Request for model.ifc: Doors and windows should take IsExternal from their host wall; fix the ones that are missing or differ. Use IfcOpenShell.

First a look at what the model holds.

```python
import ifcopenshell
import ifcopenshell.util.element

model = ifcopenshell.open("model.ifc")
print(model.schema)
seen = {}
for e in model.by_type("IfcDoor") + model.by_type("IfcWindow"):
    if not e.FillsVoids:
        continue
    host = e.FillsVoids[0].RelatingOpeningElement.VoidsElements[0].RelatingBuildingElement
    own = ifcopenshell.util.element.get_pset(e, f"Pset_{e.is_a()[3:].removesuffix('StandardCase')}Common", "IsExternal")
    wall = ifcopenshell.util.element.get_pset(host, "Pset_WallCommon", "IsExternal")
    seen[e.is_a(), own, wall] = seen.get((e.is_a(), own, wall), 0) + 1
for (cls, own, wall), count in sorted(seen.items(), key=str):
    print(count, cls, "IsExternal:", own, "| host wall:", wall)
```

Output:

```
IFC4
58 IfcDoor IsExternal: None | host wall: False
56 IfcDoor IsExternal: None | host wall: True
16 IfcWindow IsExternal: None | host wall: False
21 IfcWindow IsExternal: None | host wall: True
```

```python
import ifcopenshell
import ifcopenshell.api.pset
import ifcopenshell.util.element

model = ifcopenshell.open("model.ifc")

count = 0
for ifc_class, pset_name in (("IfcDoor", "Pset_DoorCommon"), ("IfcWindow", "Pset_WindowCommon")):
    for e in model.by_type(ifc_class):
        if not e.FillsVoids:
            continue
        host = e.FillsVoids[0].RelatingOpeningElement.VoidsElements[0].RelatingBuildingElement
        external = ifcopenshell.util.element.get_pset(host, "Pset_WallCommon", "IsExternal")
        if external is None or ifcopenshell.util.element.get_pset(e, pset_name, "IsExternal") == external:
            continue
        pset = ifcopenshell.api.pset.add_pset(model, product=e, name=pset_name)
        ifcopenshell.api.pset.edit_pset(model, pset=pset, properties={"IsExternal": external})
        count += 1

print(count, "updated")

model.write("model_v2.ifc")
```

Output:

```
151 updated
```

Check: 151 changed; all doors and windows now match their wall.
